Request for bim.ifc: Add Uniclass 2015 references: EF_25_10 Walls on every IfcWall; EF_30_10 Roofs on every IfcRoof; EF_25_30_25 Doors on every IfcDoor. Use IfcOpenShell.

First a look at what the model holds.

```python
import ifcopenshell

model = ifcopenshell.open("bim.ifc")
print(model.schema)
print("classifications:", [c.Name for c in model.by_type("IfcClassification")])
for ifc_class in ("IfcDoor", "IfcRoof", "IfcStair", "IfcWall", "IfcWindow"):
    print(ifc_class, len(model.by_type(ifc_class)))
```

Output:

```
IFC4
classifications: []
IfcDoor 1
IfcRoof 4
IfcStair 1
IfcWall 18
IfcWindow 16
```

```python
import ifcopenshell
import ifcopenshell.api.classification

model = ifcopenshell.open("bim.ifc")

system = ifcopenshell.api.classification.add_classification(model, classification="Uniclass 2015")

codes = {
    "IfcWall": ("EF_25_10", "Walls"),
    "IfcRoof": ("EF_30_10", "Roofs"),
    "IfcDoor": ("EF_25_30_25", "Doors"),
}
for ifc_class, (code, name) in codes.items():
    products = model.by_type(ifc_class)
    ifcopenshell.api.classification.add_reference(
        model, products=products, classification=system, identification=code, name=name
    )
    print(code, len(products))

model.write("bim_v2.ifc")
```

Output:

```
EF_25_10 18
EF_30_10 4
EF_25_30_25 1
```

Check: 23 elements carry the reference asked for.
